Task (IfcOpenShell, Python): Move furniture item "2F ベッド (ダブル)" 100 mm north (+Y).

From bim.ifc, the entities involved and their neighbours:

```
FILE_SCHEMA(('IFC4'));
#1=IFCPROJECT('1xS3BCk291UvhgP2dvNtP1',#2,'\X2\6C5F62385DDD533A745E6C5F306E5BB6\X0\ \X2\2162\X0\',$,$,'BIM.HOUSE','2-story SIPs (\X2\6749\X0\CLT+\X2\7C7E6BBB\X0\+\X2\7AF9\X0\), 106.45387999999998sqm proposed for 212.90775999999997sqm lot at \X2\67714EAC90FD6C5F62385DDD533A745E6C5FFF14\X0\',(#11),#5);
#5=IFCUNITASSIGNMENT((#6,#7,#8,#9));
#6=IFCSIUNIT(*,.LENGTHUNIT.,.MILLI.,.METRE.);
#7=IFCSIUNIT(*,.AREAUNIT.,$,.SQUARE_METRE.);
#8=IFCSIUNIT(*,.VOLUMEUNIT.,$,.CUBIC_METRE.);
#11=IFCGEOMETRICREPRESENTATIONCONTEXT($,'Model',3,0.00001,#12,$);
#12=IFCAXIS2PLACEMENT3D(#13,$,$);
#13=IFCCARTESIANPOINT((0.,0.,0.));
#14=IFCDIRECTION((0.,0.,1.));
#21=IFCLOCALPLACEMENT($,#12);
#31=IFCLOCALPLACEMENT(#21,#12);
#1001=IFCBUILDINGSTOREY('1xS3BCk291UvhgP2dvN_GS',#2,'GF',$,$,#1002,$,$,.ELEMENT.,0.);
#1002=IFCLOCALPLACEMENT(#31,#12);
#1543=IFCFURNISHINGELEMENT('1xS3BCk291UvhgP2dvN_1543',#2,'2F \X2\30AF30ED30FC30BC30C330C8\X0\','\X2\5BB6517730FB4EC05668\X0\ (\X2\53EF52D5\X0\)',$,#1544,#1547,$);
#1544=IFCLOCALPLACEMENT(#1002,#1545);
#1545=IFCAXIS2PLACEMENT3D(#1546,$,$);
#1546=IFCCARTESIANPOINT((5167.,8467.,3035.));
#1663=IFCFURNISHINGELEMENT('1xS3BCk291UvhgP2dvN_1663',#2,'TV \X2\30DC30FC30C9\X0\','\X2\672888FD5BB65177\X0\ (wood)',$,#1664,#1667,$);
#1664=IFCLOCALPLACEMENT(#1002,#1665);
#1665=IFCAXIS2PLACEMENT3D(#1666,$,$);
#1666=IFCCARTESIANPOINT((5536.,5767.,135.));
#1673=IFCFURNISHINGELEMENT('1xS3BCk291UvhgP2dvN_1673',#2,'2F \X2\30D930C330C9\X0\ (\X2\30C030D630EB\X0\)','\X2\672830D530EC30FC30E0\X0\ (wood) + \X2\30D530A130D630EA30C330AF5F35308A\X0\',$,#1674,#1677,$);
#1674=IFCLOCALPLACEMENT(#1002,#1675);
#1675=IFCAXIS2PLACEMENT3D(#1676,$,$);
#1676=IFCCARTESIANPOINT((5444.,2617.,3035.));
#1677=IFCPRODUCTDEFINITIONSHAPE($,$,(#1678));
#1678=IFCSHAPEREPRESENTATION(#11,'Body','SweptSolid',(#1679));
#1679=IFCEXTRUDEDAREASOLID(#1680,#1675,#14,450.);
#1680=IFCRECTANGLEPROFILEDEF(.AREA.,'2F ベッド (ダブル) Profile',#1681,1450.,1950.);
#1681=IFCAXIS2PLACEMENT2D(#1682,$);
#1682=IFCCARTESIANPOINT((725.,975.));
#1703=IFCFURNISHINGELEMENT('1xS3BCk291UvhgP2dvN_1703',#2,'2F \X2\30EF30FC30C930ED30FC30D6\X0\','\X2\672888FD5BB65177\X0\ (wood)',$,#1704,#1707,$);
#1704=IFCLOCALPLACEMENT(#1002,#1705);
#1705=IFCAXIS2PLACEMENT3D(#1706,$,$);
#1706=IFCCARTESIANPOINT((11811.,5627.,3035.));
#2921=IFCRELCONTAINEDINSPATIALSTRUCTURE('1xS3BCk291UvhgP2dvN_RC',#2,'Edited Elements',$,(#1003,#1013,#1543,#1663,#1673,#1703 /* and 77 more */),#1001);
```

```python
import ifcopenshell
import ifcopenshell.api.geometry
import ifcopenshell.util.placement
import ifcopenshell.util.unit

model = ifcopenshell.open("bim.ifc")
unit_scale = ifcopenshell.util.unit.calculate_unit_scale(model)

item = model.by_guid("1xS3BCk291UvhgP2dvN_1673")
matrix = ifcopenshell.util.placement.get_local_placement(item.ObjectPlacement)
matrix[1, 3] += 0.1 / unit_scale
ifcopenshell.api.geometry.edit_object_placement(model, product=item, matrix=matrix, is_si=False)

print(ifcopenshell.util.placement.get_local_placement(item.ObjectPlacement).round(3) + 0.0)

model.write("bim_v2.ifc")
```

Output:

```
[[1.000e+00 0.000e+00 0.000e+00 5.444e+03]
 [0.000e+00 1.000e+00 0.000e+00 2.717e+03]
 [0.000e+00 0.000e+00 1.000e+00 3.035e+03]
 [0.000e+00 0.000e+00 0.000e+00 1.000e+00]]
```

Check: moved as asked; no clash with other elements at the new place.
